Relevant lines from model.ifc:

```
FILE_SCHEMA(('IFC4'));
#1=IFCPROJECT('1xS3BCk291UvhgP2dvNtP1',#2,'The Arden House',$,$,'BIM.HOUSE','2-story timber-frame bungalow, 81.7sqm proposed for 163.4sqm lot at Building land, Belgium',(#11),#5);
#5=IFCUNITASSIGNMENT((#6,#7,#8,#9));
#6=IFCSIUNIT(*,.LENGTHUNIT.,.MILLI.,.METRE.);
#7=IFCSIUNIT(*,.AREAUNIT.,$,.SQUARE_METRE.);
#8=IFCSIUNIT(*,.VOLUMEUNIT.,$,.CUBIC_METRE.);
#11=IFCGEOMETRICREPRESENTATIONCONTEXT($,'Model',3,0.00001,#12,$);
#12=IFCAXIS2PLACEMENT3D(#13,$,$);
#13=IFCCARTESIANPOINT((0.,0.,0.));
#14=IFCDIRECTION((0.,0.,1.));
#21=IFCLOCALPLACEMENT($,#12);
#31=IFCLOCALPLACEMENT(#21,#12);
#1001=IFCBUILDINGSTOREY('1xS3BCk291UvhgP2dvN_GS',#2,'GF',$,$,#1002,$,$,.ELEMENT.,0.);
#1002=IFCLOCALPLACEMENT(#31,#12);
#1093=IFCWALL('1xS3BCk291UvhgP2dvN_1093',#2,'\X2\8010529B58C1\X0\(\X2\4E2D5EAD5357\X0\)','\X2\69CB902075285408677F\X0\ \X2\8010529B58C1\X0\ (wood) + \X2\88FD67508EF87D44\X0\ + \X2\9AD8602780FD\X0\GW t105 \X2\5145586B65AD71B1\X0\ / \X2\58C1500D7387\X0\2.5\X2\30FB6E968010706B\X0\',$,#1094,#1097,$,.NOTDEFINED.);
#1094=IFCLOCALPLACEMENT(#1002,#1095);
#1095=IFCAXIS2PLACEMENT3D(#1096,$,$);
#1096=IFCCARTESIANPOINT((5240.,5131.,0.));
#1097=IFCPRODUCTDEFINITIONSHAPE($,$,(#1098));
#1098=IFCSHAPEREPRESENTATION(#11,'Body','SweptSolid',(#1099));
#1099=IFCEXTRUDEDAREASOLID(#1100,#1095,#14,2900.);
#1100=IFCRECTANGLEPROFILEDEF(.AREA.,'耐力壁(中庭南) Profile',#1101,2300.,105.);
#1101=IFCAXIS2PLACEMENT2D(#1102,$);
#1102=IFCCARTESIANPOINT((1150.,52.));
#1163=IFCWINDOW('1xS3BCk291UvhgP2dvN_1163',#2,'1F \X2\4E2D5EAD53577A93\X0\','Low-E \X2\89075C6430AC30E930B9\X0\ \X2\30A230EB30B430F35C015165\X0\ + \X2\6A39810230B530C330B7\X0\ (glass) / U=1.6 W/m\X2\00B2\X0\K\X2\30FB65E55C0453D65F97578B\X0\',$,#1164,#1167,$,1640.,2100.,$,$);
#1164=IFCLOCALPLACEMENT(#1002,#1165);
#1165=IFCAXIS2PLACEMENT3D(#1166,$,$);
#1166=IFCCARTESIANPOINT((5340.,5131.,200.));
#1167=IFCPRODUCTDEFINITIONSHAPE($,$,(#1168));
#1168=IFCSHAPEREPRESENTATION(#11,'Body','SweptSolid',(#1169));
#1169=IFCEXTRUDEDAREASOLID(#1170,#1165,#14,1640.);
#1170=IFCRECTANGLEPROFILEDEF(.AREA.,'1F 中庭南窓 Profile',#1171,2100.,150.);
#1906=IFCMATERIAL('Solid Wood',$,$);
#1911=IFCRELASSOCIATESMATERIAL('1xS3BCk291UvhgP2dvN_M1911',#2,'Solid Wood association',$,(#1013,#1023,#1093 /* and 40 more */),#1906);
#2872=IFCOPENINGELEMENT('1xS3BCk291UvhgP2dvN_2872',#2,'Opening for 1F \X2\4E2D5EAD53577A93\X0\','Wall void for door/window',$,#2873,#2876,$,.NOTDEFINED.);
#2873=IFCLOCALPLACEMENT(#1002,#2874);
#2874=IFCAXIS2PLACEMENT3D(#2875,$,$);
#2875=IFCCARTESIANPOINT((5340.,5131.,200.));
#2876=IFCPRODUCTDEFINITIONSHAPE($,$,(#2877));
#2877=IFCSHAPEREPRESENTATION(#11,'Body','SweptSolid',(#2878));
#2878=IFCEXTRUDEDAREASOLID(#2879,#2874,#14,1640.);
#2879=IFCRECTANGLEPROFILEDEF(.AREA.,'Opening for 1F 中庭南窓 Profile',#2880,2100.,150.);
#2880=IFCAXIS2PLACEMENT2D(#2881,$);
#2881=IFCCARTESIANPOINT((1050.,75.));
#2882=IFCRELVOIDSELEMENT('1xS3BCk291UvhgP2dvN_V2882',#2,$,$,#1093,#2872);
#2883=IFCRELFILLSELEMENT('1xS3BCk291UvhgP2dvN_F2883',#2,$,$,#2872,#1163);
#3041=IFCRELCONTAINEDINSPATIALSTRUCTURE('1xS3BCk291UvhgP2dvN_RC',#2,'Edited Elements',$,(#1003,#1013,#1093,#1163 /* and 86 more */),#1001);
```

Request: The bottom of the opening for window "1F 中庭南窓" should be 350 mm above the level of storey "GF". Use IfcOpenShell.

```python
import numpy as np
import ifcopenshell
import ifcopenshell.api.geometry
import ifcopenshell.geom
import ifcopenshell.util.element
import ifcopenshell.util.placement
import ifcopenshell.util.shape
import ifcopenshell.util.unit

model = ifcopenshell.open("model.ifc")
unit_scale = ifcopenshell.util.unit.calculate_unit_scale(model)

window = model.by_guid("1xS3BCk291UvhgP2dvN_1163")
opening = window.FillsVoids[0].RelatingOpeningElement
storey = ifcopenshell.util.element.get_container(window, ifc_class="IfcBuildingStorey")
level = ifcopenshell.util.placement.get_local_placement(storey.ObjectPlacement)[2, 3]

# The opening's origin need not be at the sill, so measure its lowest point.
shape = ifcopenshell.geom.create_shape(ifcopenshell.geom.settings(), opening)
bottom = ifcopenshell.util.shape.get_shape_bottom_elevation(shape, shape.geometry) / unit_scale
dz = level + 0.35 / unit_scale - bottom

shift = np.array([0.0, 0.0, dz])
# The window is not placed relative to its opening, so move both.
for product in (opening, window):
    matrix = ifcopenshell.util.placement.get_local_placement(product.ObjectPlacement)
    matrix[:3, 3] += shift
    ifcopenshell.api.geometry.edit_object_placement(model, product=product, matrix=matrix, is_si=False)

print(f"moved by {dz * unit_scale:+.3f} m")

model.write("model_v2.ifc")
```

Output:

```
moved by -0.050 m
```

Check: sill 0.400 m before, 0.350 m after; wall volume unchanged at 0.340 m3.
